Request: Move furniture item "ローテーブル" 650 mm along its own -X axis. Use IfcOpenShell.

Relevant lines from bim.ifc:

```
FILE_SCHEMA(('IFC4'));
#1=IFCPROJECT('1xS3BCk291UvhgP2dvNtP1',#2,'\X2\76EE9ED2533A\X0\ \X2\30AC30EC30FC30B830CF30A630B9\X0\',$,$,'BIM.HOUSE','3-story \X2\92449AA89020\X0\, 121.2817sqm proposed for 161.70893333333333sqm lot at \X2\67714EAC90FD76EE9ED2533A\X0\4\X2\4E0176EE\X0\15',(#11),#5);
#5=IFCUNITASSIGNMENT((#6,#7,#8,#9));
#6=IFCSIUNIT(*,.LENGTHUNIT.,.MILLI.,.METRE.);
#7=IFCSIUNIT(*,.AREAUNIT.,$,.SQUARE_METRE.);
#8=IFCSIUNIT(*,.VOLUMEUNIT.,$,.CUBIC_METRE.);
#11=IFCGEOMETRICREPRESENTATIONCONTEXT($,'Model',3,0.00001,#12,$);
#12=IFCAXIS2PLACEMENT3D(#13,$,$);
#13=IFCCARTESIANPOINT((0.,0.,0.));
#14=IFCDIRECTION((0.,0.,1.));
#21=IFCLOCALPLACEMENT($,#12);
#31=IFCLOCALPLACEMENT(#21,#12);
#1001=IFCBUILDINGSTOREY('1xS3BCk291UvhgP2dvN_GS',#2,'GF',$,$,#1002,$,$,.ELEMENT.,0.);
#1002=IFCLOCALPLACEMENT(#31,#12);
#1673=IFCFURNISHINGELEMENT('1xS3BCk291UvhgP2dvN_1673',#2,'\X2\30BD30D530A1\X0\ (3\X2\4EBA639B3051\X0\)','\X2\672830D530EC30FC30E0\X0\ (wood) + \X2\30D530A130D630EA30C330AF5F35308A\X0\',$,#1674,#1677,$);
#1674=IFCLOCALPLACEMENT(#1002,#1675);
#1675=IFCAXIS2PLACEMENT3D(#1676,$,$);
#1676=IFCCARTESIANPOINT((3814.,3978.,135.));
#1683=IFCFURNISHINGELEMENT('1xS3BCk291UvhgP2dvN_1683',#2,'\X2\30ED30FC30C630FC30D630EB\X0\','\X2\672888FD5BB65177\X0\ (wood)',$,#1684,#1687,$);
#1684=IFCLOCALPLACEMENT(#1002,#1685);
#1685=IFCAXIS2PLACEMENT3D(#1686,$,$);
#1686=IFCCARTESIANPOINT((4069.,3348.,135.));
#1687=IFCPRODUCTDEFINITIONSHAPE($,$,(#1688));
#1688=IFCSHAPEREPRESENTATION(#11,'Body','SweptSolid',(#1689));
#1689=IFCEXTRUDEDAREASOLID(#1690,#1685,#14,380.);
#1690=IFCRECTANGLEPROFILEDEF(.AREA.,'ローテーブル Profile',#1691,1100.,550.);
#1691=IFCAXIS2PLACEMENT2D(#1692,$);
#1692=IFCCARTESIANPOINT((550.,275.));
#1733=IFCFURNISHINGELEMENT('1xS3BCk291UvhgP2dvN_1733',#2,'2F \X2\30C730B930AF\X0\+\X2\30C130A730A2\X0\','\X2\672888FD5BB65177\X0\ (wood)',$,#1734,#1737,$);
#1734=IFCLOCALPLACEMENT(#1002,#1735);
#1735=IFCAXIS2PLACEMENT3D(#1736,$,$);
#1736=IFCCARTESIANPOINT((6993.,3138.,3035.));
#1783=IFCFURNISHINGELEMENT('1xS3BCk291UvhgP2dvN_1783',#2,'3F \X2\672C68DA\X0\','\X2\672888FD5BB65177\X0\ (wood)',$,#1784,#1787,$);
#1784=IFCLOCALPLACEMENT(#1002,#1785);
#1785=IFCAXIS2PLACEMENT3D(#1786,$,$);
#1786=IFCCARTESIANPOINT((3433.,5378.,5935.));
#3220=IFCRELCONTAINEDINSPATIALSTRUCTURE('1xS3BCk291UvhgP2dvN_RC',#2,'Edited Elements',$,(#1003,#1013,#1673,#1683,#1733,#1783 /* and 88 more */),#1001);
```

```python
import ifcopenshell
import ifcopenshell.api.geometry
import ifcopenshell.util.placement
import ifcopenshell.util.unit

model = ifcopenshell.open("bim.ifc")
unit_scale = ifcopenshell.util.unit.calculate_unit_scale(model)

item = model.by_guid("1xS3BCk291UvhgP2dvN_1683")
matrix = ifcopenshell.util.placement.get_local_placement(item.ObjectPlacement)
matrix[:3, 3] -= matrix[:3, 0] * 0.65 / unit_scale
ifcopenshell.api.geometry.edit_object_placement(model, product=item, matrix=matrix, is_si=False)

print(ifcopenshell.util.placement.get_local_placement(item.ObjectPlacement).round(3) + 0.0)

model.write("bim_rev.ifc")
```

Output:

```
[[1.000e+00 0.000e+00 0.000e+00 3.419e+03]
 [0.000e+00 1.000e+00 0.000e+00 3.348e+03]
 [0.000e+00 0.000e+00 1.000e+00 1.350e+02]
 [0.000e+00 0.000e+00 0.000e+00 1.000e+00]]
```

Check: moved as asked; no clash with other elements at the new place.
